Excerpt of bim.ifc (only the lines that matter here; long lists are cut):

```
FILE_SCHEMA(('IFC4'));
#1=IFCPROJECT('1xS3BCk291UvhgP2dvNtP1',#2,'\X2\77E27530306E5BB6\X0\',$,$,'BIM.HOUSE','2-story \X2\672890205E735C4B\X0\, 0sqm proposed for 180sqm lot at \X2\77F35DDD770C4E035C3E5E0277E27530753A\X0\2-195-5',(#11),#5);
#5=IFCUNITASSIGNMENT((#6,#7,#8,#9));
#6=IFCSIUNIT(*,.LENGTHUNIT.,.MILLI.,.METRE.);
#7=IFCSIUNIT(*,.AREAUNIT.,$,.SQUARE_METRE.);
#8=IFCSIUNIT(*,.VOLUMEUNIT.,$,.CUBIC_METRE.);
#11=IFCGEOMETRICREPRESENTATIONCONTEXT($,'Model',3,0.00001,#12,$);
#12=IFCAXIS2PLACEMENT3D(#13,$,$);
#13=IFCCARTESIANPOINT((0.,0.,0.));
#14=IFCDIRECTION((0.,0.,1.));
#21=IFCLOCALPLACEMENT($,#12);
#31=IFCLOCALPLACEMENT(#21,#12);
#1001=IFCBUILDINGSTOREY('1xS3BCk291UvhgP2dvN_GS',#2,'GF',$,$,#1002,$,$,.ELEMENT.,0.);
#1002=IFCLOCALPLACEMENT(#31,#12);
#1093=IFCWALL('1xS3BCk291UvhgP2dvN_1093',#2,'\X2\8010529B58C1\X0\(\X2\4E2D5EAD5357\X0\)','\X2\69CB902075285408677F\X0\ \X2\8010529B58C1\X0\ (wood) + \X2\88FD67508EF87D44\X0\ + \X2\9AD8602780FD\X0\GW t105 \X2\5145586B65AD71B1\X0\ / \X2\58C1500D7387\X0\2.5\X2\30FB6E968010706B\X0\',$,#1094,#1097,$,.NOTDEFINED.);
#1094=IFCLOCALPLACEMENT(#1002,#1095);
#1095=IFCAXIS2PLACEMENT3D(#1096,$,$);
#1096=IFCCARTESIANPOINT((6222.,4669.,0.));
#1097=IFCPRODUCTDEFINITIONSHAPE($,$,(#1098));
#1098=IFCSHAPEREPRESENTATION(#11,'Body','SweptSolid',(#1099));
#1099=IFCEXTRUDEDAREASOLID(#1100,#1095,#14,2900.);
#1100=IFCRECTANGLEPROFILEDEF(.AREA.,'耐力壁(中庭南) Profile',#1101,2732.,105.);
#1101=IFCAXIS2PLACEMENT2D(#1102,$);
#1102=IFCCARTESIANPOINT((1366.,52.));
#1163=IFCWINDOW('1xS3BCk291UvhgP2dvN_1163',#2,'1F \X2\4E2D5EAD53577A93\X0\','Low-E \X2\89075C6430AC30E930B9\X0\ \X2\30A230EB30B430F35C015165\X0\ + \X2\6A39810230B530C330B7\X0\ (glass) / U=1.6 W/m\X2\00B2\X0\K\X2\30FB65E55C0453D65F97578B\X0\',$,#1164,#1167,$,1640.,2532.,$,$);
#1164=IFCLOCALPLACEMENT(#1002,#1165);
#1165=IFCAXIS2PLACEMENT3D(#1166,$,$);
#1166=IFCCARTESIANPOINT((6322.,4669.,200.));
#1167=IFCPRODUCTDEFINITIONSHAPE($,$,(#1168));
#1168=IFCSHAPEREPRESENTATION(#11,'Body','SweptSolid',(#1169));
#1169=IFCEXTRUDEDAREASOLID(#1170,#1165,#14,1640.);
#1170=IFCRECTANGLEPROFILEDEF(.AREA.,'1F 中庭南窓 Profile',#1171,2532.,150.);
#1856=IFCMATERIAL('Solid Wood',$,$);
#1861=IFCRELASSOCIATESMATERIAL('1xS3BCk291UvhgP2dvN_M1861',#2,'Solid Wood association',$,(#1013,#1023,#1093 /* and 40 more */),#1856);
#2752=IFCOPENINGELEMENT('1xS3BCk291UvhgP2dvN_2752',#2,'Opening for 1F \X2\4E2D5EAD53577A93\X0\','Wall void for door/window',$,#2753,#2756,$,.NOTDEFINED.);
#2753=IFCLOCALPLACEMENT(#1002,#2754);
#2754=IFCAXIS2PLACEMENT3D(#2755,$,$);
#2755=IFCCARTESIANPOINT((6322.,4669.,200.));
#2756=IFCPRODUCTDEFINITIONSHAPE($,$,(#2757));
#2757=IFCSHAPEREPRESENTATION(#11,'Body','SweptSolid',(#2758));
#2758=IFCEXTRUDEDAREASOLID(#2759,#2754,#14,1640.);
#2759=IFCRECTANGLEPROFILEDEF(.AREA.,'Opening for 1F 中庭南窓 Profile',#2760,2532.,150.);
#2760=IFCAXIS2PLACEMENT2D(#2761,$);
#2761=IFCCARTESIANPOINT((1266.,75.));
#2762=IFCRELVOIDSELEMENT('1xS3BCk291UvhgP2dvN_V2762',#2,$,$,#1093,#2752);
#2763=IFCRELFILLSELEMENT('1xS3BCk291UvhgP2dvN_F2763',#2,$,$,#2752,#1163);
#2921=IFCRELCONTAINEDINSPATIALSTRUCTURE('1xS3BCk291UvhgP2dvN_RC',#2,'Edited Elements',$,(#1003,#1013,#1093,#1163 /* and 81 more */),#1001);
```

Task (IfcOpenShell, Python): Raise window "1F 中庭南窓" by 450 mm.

```python
import numpy as np
import ifcopenshell
import ifcopenshell.api.geometry
import ifcopenshell.util.placement
import ifcopenshell.util.unit

model = ifcopenshell.open("bim.ifc")
unit_scale = ifcopenshell.util.unit.calculate_unit_scale(model)

window = model.by_id(1163)
opening = window.FillsVoids[0].RelatingOpeningElement
dz = 450.0

shift = np.array([0.0, 0.0, dz])
# The window is not placed relative to its opening, so move both.
for product in (opening, window):
    matrix = ifcopenshell.util.placement.get_local_placement(product.ObjectPlacement)
    matrix[:3, 3] += shift
    ifcopenshell.api.geometry.edit_object_placement(model, product=product, matrix=matrix, is_si=False)

print(f"moved by {dz * unit_scale:+.3f} m")

model.write("bim_updated.ifc")
```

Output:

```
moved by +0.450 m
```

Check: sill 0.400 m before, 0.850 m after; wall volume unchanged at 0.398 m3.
